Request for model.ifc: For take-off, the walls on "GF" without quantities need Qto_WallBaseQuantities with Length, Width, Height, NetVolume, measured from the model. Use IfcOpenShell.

First a look at what the model holds.

```python
import ifcopenshell
import ifcopenshell.util.element
import ifcopenshell.util.unit

model = ifcopenshell.open("model.ifc")
print(model.schema)
for unit_type in ("LENGTHUNIT", "AREAUNIT", "VOLUMEUNIT"):
    print(unit_type, ifcopenshell.util.unit.calculate_unit_scale(model, unit_type))
storey = next(s for s in model.by_type("IfcBuildingStorey") if s.Name == "GF")
walls = [e for e in ifcopenshell.util.element.get_decomposition(storey) if e.is_a("IfcWall")]
for e in sorted(walls, key=lambda e: e.id()):
    print(e.id(), e.is_a(), e.Name, list(ifcopenshell.util.element.get_psets(e, qtos_only=True)), sep=" | ")
```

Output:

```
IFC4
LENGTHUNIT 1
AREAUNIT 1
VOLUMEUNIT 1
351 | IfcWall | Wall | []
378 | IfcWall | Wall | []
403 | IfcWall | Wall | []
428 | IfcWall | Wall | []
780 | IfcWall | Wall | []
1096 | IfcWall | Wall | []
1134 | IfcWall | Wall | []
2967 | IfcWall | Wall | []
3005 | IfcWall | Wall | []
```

```python
import ifcopenshell
import ifcopenshell.api.pset
import ifcopenshell.geom
import ifcopenshell.util.element
import ifcopenshell.util.shape
import ifcopenshell.util.unit

model = ifcopenshell.open("model.ifc")
unit_scale = ifcopenshell.util.unit.calculate_unit_scale(model)
volume_scale = ifcopenshell.util.unit.calculate_unit_scale(model, "VOLUMEUNIT")
settings = ifcopenshell.geom.settings()

storey = next(s for s in model.by_type("IfcBuildingStorey") if s.Name == "GF")
walls = [e for e in ifcopenshell.util.element.get_decomposition(storey) if e.is_a("IfcWall")]

for e in sorted(walls, key=lambda e: e.id()):
    if ifcopenshell.util.element.get_psets(e, qtos_only=True, should_inherit=False):
        continue
    # Geometry comes back in metres, in the element's own axes.
    shape = ifcopenshell.geom.create_shape(settings, e)
    values = {
        "Length": ifcopenshell.util.shape.get_x(shape.geometry) / unit_scale,
        "Width": ifcopenshell.util.shape.get_y(shape.geometry) / unit_scale,
        "Height": ifcopenshell.util.shape.get_z(shape.geometry) / unit_scale,
        "NetVolume": ifcopenshell.util.shape.get_volume(shape.geometry) / volume_scale,
    }
    qto = ifcopenshell.api.pset.add_qto(model, product=e, name="Qto_WallBaseQuantities")
    ifcopenshell.api.pset.edit_qto(model, qto=qto, properties=values)
    print(e.id(), {k: round(v, 3) for k, v in values.items()})

model.write("model_v2.ifc")
```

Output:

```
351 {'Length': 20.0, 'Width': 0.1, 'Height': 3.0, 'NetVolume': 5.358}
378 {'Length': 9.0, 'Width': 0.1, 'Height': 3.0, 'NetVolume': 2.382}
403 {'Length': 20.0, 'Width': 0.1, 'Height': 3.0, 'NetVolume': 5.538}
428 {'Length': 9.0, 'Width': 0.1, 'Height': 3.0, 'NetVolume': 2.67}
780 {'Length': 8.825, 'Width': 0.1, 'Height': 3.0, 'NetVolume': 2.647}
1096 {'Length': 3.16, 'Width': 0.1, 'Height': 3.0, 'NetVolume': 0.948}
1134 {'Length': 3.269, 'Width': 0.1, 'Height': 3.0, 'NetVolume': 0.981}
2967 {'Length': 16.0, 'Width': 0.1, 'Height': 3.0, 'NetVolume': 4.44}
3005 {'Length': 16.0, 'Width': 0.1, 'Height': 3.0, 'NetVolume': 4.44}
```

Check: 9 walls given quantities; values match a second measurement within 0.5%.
